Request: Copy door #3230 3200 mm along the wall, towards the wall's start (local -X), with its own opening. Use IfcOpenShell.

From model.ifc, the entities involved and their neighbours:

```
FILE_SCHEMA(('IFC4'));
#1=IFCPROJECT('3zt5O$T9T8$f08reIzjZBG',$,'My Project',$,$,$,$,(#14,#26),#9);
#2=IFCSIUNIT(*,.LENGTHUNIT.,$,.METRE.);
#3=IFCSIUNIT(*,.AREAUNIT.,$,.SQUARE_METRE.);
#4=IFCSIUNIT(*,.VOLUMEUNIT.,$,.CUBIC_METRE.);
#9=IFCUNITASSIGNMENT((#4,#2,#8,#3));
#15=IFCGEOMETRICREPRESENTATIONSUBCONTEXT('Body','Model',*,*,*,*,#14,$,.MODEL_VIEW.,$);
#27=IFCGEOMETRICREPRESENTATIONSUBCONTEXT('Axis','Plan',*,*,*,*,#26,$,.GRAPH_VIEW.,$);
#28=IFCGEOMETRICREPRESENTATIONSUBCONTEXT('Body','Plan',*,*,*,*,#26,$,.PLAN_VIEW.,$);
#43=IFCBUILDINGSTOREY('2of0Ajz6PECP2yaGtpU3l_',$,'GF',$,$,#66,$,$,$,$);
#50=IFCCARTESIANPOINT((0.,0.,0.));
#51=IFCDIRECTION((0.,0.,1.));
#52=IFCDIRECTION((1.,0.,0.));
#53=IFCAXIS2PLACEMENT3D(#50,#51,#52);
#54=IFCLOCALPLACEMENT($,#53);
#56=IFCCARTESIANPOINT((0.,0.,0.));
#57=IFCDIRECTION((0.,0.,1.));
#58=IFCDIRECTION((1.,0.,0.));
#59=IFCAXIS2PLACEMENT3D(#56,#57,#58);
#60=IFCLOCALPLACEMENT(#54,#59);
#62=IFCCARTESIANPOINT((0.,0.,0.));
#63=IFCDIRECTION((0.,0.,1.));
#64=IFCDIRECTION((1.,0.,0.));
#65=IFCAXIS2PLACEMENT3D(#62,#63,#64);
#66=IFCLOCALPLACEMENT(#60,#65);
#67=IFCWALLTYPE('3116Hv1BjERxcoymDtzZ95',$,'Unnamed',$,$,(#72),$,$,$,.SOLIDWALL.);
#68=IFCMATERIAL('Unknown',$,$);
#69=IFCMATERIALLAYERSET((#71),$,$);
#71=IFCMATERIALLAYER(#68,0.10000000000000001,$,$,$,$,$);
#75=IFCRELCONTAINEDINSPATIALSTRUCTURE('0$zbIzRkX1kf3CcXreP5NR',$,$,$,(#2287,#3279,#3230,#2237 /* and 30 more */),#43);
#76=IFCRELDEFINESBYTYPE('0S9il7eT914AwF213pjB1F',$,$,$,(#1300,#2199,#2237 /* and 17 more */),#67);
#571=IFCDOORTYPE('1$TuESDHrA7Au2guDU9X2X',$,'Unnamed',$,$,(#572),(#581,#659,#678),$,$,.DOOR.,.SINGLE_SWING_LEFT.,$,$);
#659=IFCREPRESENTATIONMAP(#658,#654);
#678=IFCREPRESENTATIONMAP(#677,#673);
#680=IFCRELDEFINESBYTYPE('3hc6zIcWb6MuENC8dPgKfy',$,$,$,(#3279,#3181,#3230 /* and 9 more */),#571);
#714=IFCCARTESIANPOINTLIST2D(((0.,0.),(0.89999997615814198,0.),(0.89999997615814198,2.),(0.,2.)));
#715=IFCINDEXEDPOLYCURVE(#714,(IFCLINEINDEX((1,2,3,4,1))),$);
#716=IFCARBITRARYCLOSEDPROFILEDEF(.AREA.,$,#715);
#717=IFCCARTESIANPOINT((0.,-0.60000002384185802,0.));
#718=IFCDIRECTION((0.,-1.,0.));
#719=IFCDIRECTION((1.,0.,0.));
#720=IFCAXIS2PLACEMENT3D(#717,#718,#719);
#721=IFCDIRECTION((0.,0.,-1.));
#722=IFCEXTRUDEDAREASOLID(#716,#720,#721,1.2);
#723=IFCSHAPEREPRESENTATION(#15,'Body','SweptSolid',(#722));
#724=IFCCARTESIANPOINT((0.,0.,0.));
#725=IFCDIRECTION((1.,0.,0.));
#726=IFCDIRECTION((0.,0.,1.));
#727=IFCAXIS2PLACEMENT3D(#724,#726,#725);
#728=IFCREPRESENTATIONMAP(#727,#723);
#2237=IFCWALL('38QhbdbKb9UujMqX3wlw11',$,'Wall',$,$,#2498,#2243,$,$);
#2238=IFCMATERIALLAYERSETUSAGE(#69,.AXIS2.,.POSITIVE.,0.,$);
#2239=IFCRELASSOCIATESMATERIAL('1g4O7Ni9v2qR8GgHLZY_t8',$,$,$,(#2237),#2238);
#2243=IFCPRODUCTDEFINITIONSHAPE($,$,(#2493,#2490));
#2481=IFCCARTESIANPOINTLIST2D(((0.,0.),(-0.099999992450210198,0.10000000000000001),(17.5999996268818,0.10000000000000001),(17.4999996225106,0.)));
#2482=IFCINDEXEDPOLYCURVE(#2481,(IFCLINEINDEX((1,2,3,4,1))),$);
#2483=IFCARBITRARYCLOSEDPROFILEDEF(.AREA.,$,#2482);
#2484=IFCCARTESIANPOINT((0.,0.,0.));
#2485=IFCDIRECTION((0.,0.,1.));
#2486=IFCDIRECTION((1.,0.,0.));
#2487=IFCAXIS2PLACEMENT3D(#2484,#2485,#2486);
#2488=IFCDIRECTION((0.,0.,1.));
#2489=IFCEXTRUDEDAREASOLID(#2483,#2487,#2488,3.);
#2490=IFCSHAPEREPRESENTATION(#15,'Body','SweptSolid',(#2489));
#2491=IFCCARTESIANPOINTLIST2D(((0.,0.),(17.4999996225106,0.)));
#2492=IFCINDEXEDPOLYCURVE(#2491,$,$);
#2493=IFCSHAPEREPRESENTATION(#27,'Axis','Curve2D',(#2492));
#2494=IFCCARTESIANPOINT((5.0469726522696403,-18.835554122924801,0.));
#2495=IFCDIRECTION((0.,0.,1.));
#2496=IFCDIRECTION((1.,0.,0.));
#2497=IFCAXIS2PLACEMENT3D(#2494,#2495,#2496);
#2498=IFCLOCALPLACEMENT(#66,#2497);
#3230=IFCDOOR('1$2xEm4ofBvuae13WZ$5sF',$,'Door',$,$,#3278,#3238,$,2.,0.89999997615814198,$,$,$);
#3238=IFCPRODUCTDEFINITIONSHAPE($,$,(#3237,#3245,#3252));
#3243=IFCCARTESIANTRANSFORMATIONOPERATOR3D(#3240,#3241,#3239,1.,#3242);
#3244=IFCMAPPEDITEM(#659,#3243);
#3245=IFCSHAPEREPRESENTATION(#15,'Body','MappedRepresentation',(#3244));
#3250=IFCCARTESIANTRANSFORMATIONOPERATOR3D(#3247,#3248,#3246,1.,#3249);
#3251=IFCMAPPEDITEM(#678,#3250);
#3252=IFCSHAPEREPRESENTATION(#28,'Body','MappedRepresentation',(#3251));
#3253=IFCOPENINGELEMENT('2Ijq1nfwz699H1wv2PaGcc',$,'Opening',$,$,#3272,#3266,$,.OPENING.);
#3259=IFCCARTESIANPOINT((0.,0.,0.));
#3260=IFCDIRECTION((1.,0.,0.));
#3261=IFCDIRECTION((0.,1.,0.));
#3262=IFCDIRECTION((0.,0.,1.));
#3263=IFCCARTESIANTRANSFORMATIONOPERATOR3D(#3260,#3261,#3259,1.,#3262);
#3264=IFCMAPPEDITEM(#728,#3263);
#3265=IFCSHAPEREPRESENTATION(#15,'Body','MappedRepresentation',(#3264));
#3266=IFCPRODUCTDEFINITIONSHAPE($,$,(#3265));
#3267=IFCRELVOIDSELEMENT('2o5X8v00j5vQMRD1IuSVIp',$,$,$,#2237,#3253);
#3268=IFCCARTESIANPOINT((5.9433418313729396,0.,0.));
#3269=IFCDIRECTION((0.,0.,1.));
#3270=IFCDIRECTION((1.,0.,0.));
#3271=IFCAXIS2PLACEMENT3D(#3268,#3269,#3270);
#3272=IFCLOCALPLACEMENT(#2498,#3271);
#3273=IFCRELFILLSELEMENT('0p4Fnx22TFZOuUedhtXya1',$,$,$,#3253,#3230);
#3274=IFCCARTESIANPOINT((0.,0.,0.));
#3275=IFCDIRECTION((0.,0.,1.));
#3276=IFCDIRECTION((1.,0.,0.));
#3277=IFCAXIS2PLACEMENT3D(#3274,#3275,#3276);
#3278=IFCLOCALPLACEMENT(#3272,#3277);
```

```python
import ifcopenshell
import ifcopenshell.api.feature
import ifcopenshell.api.geometry
import ifcopenshell.api.root
import ifcopenshell.geom
import ifcopenshell.util.element
import ifcopenshell.util.placement
import ifcopenshell.util.shape

model = ifcopenshell.open("model.ifc")
settings = ifcopenshell.geom.settings()


def volume(element):
    """Net volume in cubic metres, openings subtracted."""
    shape = ifcopenshell.geom.create_shape(settings, element)
    return ifcopenshell.util.shape.get_volume(shape.geometry)


door = model.by_id(3230)
opening = door.FillsVoids[0].RelatingOpeningElement
wall = opening.VoidsElements[0].RelatingBuildingElement
before = volume(wall)
shift = ifcopenshell.util.placement.get_local_placement(wall.ObjectPlacement)[:3, 0] * -3.2

# copy_class copies the void relationship, type, container and properties, but no geometry.
new_opening = ifcopenshell.api.root.copy_class(model, product=opening)
new_opening.Representation = ifcopenshell.util.element.copy_deep(
    model, opening.Representation, exclude=["IfcGeometricRepresentationContext", "IfcRepresentationMap"]
)
new_door = ifcopenshell.api.root.copy_class(model, product=door)
new_door.Representation = ifcopenshell.util.element.copy_deep(
    model, door.Representation, exclude=["IfcGeometricRepresentationContext", "IfcRepresentationMap"]
)
ifcopenshell.api.feature.add_filling(model, opening=new_opening, element=new_door)

for old, new in ((opening, new_opening), (door, new_door)):
    matrix = ifcopenshell.util.placement.get_local_placement(old.ObjectPlacement)
    matrix[:3, 3] += shift
    ifcopenshell.api.geometry.edit_object_placement(model, product=new, matrix=matrix, is_si=False)

after = volume(wall)

print(f"wall volume {before:.3f} -> {after:.3f} m3")

model.write("model_edited.ifc")
```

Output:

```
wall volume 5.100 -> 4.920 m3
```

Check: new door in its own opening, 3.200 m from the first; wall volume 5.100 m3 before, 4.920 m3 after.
